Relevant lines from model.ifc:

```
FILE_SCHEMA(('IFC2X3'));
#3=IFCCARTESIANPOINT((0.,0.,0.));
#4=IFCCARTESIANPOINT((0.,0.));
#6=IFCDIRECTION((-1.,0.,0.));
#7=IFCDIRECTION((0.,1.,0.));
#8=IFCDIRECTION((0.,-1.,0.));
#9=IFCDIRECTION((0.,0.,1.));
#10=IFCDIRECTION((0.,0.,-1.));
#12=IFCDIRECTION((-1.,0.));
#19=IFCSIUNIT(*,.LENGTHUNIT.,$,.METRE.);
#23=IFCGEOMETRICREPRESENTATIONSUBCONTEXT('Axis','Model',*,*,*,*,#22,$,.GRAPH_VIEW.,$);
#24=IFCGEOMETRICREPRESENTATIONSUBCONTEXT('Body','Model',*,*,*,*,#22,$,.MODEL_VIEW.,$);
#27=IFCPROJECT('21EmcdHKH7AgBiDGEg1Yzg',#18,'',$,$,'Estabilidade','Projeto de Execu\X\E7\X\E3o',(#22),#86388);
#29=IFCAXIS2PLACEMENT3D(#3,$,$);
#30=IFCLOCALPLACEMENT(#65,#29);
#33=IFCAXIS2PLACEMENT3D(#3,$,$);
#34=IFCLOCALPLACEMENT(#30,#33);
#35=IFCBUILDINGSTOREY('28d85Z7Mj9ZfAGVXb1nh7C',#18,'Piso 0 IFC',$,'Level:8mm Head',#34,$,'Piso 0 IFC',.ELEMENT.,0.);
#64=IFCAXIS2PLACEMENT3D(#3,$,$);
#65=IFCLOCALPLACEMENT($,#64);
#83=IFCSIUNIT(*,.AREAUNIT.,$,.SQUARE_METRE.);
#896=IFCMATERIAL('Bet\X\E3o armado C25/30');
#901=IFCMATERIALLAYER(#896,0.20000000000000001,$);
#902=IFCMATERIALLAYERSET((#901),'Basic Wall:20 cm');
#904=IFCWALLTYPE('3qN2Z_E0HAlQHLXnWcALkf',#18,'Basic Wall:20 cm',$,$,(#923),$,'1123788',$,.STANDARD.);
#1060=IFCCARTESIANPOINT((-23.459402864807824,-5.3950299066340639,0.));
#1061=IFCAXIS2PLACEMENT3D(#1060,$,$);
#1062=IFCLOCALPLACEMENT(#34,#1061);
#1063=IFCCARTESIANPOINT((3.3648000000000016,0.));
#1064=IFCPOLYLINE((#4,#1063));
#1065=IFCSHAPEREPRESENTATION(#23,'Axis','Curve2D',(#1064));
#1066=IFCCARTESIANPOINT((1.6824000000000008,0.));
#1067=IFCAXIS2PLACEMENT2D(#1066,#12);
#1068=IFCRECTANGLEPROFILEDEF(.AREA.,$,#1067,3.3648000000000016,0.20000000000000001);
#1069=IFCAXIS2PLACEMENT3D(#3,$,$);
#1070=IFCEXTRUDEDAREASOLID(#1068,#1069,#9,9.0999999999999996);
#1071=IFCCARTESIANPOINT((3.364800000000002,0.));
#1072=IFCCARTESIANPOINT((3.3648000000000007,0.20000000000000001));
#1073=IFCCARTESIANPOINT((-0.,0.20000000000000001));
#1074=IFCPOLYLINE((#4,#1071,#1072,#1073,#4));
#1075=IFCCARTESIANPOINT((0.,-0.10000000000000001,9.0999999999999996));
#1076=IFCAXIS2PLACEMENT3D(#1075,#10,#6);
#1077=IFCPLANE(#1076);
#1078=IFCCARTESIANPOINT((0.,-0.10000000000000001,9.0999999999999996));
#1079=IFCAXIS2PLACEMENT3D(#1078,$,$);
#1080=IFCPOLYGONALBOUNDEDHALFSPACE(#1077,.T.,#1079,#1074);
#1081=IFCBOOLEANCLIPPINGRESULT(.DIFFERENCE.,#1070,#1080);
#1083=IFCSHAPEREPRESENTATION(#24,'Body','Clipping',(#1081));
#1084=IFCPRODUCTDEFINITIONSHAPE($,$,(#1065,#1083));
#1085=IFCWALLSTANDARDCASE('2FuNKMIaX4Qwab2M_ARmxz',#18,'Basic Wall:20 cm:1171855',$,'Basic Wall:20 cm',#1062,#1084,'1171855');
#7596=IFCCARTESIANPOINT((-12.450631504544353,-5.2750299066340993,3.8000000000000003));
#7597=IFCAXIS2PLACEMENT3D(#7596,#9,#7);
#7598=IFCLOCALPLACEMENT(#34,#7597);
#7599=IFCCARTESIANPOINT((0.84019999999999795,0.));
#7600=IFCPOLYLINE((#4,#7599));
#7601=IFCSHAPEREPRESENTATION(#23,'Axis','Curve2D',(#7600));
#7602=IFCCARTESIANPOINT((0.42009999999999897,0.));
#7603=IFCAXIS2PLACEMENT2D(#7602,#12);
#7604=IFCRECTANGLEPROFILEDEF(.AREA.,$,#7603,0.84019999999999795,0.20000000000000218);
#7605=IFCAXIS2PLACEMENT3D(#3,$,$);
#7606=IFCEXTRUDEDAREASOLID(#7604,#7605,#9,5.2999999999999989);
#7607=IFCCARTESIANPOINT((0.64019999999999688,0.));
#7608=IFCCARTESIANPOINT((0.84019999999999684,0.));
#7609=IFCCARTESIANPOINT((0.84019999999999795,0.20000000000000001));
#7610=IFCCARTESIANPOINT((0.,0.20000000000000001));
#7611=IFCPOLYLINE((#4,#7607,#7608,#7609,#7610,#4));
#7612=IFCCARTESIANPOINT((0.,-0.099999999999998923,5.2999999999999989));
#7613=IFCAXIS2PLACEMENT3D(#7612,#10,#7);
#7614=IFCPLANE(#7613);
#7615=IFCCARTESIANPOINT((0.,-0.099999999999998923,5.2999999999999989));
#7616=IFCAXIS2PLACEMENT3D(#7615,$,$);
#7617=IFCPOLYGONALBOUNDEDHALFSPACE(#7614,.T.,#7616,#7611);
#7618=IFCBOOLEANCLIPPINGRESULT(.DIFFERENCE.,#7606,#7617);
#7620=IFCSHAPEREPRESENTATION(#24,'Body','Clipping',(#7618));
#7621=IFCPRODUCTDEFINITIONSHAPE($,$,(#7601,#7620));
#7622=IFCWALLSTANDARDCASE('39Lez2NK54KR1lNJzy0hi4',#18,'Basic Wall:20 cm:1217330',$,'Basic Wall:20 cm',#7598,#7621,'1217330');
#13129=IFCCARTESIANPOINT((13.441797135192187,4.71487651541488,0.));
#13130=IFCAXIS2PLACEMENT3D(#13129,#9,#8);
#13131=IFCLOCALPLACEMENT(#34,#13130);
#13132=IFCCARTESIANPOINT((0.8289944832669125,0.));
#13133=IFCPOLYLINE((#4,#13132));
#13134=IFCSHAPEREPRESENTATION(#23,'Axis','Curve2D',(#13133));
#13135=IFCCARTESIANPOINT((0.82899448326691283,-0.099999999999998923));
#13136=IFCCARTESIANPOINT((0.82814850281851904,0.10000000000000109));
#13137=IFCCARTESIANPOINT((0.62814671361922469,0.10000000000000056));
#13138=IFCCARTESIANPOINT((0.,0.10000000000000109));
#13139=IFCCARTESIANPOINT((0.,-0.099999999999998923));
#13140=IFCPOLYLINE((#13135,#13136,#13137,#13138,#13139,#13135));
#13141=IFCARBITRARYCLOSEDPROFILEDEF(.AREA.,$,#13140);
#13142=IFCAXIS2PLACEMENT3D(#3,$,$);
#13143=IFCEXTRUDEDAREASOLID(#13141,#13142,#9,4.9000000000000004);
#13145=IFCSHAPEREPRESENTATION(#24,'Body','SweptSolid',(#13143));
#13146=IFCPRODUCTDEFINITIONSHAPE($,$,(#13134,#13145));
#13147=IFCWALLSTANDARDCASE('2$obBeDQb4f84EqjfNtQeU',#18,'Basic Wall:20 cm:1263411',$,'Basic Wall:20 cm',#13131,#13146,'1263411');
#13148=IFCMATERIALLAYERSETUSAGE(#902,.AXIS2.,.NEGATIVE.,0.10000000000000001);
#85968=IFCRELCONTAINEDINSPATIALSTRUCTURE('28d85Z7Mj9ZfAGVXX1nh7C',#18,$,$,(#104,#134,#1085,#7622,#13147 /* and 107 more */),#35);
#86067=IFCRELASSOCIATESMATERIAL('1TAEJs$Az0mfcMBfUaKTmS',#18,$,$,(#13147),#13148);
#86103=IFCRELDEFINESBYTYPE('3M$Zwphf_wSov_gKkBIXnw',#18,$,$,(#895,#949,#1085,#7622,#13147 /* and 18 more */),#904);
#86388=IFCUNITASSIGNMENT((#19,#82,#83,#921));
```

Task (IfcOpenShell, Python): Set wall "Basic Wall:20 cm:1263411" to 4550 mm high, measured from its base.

```python
import ifcopenshell
import ifcopenshell.geom
import ifcopenshell.util.representation
import ifcopenshell.util.shape

model = ifcopenshell.open("model.ifc")
settings = ifcopenshell.geom.settings()


def volume(element):
    """Net volume in cubic metres, openings subtracted."""
    shape = ifcopenshell.geom.create_shape(settings, element)
    return ifcopenshell.util.shape.get_volume(shape.geometry)


wall = model.by_guid("2$obBeDQb4f84EqjfNtQeU")
before = volume(wall)

body = ifcopenshell.util.representation.get_representation(wall, "Model", "Body")
solid = body.Items[0]
old_height = solid.Depth
solid.Depth = 4.55
after = volume(wall)

print(f"height {old_height:g} -> {solid.Depth:g}, volume {before:.3f} -> {after:.3f} m3")

model.write("model_updated.ifc")
```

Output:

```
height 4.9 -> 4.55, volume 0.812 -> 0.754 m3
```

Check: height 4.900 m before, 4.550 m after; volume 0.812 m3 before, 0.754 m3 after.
